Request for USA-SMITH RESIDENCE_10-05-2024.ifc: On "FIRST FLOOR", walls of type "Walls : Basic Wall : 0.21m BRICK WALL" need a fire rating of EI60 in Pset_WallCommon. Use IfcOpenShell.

First a look at what the model holds.

```python
import ifcopenshell
import ifcopenshell.util.element

model = ifcopenshell.open("USA-SMITH RESIDENCE_10-05-2024.ifc")
print(model.schema)
storey = next(s for s in model.by_type("IfcBuildingStorey") if s.Name == "FIRST FLOOR")
walls = [e for e in ifcopenshell.util.element.get_decomposition(storey) if e.is_a("IfcWall")]
seen = {}
for e in walls:
    element_type = ifcopenshell.util.element.get_type(e)
    key = (element_type.Name if element_type != e and element_type else None, ifcopenshell.util.element.get_pset(e, "Pset_WallCommon", "FireRating"))
    seen[key] = seen.get(key, 0) + 1
for (name, value), count in sorted(seen.items(), key=str):
    print(count, "x", name, "|", value)
```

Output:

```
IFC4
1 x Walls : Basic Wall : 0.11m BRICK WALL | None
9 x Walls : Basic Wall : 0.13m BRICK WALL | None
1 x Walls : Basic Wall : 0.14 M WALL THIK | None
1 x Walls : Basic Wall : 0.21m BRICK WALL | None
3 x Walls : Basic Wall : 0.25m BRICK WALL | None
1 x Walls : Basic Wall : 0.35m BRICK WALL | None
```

```python
import ifcopenshell
import ifcopenshell.api.pset
import ifcopenshell.util.element

model = ifcopenshell.open("USA-SMITH RESIDENCE_10-05-2024.ifc")

storey = next(s for s in model.by_type("IfcBuildingStorey") if s.Name == "FIRST FLOOR")
walls = [e for e in ifcopenshell.util.element.get_decomposition(storey) if e.is_a("IfcWall")]

count = 0
for e in walls:
    element_type = ifcopenshell.util.element.get_type(e)
    if element_type in (None, e) or element_type.Name != "Walls : Basic Wall : 0.21m BRICK WALL":
        continue
    # add_pset returns the element's existing set when there is one.
    pset = ifcopenshell.api.pset.add_pset(model, product=e, name="Pset_WallCommon")
    ifcopenshell.api.pset.edit_pset(model, pset=pset, properties={"FireRating": "EI60"})
    count += 1

print(count, "walls updated")

model.write("USA-SMITH RESIDENCE_10-05-2024-out.ifc")
```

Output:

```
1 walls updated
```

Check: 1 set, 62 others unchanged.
